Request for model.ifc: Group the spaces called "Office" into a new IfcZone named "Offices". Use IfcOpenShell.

First a look at what the model holds.

```python
import ifcopenshell

model = ifcopenshell.open("model.ifc")
print(model.schema)
seen = {}
for space in model.by_type("IfcSpace"):
    seen[space.LongName] = seen.get(space.LongName, 0) + 1
for name, count in sorted(seen.items(), key=str):
    print(count, "x", name)
print("zones:", [z.Name for z in model.by_type("IfcZone")][:20])
```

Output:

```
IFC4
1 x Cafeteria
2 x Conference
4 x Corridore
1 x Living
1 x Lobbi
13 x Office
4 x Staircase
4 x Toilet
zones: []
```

```python
import ifcopenshell
import ifcopenshell.api.group
import ifcopenshell.api.root

model = ifcopenshell.open("model.ifc")

names = {"Office"}
spaces = [s for s in model.by_type("IfcSpace") if s.LongName in names]

zone = ifcopenshell.api.root.create_entity(model, ifc_class="IfcZone", name="Offices")
ifcopenshell.api.group.assign_group(model, products=spaces, group=zone)
print(len(spaces), "spaces in", zone.Name)

model.write("model_v2.ifc")
```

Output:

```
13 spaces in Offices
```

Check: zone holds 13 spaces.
